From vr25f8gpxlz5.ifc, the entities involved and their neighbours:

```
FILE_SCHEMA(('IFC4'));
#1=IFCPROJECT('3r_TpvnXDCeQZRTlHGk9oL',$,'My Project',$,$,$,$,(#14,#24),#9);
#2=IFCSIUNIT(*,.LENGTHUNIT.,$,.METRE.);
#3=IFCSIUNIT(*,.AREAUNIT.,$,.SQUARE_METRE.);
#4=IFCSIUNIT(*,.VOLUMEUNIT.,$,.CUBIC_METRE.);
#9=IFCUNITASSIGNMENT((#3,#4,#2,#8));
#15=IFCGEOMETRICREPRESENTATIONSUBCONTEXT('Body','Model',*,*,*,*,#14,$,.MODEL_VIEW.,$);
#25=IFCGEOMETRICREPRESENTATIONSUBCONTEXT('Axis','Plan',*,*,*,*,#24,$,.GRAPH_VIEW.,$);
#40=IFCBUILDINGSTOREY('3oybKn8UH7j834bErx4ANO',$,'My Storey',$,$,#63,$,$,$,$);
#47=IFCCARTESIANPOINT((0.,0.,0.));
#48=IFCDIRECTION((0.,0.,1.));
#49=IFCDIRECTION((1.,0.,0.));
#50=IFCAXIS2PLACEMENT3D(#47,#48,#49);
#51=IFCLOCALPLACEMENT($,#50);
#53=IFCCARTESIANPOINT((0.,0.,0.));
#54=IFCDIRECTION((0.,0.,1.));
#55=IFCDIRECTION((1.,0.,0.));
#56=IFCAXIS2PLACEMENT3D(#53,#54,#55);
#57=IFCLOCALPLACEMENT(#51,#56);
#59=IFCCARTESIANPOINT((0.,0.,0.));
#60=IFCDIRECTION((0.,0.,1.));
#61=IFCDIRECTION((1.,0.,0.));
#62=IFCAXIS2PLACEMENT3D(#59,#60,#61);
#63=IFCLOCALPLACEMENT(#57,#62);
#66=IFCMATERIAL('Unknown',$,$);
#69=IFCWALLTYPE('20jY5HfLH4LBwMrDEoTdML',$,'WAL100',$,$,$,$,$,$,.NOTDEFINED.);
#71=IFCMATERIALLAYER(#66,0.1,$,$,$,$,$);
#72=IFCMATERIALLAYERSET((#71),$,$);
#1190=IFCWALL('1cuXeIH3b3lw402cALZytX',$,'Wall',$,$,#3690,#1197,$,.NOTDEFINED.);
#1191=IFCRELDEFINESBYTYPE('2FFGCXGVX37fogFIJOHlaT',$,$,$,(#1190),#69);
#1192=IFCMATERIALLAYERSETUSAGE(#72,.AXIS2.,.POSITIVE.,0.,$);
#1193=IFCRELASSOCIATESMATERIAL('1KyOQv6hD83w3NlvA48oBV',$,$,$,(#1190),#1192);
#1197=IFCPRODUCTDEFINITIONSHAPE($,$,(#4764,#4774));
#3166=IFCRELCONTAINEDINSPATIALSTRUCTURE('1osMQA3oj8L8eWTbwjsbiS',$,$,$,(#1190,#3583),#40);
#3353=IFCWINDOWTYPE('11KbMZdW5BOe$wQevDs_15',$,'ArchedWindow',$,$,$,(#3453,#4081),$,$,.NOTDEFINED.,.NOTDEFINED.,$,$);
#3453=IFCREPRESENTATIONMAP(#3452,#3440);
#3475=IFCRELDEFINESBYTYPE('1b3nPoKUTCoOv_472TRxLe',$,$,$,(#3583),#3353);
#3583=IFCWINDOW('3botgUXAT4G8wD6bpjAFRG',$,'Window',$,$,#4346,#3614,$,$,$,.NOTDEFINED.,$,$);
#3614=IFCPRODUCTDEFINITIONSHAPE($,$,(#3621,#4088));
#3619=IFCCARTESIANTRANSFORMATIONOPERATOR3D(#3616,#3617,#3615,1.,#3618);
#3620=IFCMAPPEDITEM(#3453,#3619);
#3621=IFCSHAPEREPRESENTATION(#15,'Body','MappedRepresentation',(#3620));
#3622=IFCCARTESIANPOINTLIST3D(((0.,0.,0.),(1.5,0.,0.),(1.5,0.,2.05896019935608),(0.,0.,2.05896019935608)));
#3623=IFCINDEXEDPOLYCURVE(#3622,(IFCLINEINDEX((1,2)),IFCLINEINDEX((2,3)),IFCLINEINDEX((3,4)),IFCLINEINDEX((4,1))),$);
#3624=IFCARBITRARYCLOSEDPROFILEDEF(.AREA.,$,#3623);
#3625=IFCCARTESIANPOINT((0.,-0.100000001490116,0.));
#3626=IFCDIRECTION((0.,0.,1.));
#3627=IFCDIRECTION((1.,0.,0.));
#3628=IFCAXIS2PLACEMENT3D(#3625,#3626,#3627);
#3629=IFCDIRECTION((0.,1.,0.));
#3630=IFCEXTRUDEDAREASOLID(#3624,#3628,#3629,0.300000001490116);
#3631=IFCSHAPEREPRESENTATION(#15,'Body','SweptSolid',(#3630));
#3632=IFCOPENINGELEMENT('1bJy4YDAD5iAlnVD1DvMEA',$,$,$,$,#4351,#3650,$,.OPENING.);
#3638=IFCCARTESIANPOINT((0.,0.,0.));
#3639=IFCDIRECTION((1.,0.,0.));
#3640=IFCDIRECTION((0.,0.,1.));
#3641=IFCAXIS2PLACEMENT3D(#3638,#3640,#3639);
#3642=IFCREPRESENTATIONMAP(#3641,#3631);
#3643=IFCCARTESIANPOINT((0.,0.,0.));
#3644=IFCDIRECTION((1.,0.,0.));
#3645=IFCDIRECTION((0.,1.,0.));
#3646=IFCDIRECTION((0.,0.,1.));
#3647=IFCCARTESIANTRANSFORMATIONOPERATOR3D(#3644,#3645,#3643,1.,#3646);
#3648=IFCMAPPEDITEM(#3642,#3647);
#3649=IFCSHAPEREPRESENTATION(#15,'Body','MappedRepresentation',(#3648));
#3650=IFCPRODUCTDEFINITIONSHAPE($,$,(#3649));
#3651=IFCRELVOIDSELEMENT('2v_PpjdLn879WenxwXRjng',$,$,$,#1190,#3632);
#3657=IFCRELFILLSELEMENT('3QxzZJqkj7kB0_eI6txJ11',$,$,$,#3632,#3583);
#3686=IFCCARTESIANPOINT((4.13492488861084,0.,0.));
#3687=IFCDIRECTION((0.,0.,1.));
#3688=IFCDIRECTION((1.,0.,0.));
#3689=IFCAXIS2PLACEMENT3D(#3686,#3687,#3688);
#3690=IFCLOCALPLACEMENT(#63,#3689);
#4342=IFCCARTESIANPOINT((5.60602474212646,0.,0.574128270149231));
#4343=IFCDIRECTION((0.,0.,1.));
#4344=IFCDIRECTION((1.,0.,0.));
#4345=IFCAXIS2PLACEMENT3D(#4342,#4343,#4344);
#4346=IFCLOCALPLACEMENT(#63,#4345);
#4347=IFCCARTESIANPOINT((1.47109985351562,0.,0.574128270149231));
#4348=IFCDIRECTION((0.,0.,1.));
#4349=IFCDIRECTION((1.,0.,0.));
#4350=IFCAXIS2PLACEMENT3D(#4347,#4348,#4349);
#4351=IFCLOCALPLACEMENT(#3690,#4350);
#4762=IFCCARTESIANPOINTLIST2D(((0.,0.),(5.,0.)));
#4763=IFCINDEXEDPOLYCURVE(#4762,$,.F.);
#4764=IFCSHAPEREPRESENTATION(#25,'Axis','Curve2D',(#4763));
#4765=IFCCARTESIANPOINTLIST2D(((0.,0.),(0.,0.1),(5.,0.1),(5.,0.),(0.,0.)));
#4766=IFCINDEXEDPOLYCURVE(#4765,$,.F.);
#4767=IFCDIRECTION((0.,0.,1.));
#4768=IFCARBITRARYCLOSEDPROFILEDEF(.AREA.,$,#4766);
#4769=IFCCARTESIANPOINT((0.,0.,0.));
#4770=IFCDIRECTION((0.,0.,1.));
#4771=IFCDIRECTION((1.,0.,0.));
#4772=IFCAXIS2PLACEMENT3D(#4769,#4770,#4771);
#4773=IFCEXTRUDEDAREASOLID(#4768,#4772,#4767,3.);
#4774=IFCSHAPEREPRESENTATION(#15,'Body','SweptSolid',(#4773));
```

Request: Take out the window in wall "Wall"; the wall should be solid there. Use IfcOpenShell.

```python
import ifcopenshell
import ifcopenshell.api.feature
import ifcopenshell.api.root
import ifcopenshell.geom
import ifcopenshell.util.shape

model = ifcopenshell.open("vr25f8gpxlz5.ifc")
settings = ifcopenshell.geom.settings()


def volume(element):
    """Net volume in cubic metres, openings subtracted."""
    shape = ifcopenshell.geom.create_shape(settings, element)
    return ifcopenshell.util.shape.get_volume(shape.geometry)


window = model.by_guid("3botgUXAT4G8wD6bpjAFRG")
opening = window.FillsVoids[0].RelatingOpeningElement
wall = opening.VoidsElements[0].RelatingBuildingElement
before = volume(wall)

ifcopenshell.api.root.remove_product(model, product=window)
ifcopenshell.api.feature.remove_feature(model, feature=opening)

after = volume(wall)

print(f"wall volume {before:.3f} -> {after:.3f} m3")

model.write("vr25f8gpxlz5_updated.ifc")
```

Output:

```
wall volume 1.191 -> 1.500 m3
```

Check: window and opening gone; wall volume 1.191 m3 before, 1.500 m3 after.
